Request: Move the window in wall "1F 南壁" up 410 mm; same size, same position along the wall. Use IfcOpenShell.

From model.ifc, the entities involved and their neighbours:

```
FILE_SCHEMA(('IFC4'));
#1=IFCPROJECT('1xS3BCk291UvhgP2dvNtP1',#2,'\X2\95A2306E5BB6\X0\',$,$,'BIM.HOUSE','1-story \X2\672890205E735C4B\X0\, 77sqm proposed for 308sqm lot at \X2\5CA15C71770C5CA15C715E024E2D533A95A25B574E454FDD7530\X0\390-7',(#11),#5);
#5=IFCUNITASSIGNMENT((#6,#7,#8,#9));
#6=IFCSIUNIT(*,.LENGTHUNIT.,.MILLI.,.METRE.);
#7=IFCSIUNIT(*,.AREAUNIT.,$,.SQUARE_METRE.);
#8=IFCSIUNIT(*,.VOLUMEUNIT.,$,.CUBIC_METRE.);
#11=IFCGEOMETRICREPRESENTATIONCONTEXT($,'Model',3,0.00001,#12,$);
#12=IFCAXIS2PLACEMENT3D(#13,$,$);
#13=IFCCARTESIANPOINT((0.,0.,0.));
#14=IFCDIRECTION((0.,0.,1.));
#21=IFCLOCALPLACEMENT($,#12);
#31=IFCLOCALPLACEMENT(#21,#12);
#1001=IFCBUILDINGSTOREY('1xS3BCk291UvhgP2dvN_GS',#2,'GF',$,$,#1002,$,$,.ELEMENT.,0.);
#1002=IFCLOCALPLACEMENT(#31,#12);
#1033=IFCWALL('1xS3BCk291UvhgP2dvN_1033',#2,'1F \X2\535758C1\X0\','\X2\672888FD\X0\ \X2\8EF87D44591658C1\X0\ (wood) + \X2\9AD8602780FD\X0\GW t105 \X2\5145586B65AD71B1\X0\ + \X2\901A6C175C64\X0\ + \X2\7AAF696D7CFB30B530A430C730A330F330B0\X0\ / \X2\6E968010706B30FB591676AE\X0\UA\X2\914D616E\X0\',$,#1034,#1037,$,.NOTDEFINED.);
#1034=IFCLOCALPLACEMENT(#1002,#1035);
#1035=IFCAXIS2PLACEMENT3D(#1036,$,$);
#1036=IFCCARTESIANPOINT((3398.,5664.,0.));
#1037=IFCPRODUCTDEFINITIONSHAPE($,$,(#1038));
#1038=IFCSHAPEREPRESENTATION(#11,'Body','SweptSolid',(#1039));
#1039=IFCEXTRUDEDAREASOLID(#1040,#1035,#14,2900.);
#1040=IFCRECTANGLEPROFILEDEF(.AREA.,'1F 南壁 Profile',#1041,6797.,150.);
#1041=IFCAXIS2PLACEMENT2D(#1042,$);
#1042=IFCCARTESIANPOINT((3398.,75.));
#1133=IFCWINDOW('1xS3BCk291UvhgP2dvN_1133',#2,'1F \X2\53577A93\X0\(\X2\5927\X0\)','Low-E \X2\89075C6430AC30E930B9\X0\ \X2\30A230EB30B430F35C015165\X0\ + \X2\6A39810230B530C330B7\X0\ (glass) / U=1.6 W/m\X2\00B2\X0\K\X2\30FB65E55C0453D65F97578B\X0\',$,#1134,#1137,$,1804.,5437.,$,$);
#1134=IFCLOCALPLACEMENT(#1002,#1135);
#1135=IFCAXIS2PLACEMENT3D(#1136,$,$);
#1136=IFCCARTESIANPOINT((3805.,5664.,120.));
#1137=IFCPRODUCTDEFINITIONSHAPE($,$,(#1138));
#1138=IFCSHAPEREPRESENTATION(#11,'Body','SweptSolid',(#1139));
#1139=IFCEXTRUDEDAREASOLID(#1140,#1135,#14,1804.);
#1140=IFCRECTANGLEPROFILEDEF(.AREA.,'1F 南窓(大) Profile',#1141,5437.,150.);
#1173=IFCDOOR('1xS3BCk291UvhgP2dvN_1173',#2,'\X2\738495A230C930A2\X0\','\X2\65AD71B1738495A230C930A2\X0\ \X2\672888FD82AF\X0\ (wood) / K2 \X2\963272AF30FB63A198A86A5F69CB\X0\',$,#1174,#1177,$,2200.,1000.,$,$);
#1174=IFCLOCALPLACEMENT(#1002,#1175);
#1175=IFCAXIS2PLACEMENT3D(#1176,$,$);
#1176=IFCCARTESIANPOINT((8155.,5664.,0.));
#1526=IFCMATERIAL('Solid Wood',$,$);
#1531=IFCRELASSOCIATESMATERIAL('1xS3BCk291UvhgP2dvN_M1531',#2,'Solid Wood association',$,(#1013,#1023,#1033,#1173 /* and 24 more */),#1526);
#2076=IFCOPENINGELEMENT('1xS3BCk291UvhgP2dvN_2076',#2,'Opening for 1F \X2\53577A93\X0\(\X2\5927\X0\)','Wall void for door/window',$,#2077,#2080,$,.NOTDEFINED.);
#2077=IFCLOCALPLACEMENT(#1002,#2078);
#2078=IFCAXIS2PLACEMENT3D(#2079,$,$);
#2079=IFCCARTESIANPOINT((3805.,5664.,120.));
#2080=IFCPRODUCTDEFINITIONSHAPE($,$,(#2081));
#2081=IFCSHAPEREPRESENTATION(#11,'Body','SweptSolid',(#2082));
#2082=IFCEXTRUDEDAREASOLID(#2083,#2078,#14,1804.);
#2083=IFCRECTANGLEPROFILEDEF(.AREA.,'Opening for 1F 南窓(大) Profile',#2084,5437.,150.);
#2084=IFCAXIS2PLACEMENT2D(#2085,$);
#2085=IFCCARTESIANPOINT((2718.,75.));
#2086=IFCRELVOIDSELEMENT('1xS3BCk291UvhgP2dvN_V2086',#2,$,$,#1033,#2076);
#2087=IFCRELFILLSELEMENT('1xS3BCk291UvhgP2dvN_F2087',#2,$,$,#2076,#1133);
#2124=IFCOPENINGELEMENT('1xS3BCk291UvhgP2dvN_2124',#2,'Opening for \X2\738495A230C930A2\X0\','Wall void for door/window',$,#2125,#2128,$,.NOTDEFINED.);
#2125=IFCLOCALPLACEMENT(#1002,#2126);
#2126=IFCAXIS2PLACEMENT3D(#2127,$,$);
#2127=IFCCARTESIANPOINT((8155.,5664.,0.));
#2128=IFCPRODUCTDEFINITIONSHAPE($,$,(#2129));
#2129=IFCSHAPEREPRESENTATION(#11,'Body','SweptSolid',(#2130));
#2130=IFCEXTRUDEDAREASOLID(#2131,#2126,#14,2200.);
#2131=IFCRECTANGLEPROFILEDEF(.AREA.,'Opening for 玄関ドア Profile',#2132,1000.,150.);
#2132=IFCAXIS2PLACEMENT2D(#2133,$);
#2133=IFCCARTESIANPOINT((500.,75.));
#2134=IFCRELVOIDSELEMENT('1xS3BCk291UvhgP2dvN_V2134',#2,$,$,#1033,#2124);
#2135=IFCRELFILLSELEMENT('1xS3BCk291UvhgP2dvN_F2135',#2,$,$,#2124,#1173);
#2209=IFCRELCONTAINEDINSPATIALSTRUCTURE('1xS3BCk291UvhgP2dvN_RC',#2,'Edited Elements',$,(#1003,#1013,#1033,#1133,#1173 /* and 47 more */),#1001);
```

```python
import numpy as np
import ifcopenshell
import ifcopenshell.api.geometry
import ifcopenshell.util.placement
import ifcopenshell.util.unit

model = ifcopenshell.open("model.ifc")
unit_scale = ifcopenshell.util.unit.calculate_unit_scale(model)

window = model.by_guid("1xS3BCk291UvhgP2dvN_1133")
opening = window.FillsVoids[0].RelatingOpeningElement
dz = 410.0

shift = np.array([0.0, 0.0, dz])
# The window is not placed relative to its opening, so move both.
for product in (opening, window):
    matrix = ifcopenshell.util.placement.get_local_placement(product.ObjectPlacement)
    matrix[:3, 3] += shift
    ifcopenshell.api.geometry.edit_object_placement(model, product=product, matrix=matrix, is_si=False)

print(f"moved by {dz * unit_scale:+.3f} m")

model.write("model_edited.ifc")
```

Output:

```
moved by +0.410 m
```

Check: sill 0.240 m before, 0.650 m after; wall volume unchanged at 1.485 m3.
